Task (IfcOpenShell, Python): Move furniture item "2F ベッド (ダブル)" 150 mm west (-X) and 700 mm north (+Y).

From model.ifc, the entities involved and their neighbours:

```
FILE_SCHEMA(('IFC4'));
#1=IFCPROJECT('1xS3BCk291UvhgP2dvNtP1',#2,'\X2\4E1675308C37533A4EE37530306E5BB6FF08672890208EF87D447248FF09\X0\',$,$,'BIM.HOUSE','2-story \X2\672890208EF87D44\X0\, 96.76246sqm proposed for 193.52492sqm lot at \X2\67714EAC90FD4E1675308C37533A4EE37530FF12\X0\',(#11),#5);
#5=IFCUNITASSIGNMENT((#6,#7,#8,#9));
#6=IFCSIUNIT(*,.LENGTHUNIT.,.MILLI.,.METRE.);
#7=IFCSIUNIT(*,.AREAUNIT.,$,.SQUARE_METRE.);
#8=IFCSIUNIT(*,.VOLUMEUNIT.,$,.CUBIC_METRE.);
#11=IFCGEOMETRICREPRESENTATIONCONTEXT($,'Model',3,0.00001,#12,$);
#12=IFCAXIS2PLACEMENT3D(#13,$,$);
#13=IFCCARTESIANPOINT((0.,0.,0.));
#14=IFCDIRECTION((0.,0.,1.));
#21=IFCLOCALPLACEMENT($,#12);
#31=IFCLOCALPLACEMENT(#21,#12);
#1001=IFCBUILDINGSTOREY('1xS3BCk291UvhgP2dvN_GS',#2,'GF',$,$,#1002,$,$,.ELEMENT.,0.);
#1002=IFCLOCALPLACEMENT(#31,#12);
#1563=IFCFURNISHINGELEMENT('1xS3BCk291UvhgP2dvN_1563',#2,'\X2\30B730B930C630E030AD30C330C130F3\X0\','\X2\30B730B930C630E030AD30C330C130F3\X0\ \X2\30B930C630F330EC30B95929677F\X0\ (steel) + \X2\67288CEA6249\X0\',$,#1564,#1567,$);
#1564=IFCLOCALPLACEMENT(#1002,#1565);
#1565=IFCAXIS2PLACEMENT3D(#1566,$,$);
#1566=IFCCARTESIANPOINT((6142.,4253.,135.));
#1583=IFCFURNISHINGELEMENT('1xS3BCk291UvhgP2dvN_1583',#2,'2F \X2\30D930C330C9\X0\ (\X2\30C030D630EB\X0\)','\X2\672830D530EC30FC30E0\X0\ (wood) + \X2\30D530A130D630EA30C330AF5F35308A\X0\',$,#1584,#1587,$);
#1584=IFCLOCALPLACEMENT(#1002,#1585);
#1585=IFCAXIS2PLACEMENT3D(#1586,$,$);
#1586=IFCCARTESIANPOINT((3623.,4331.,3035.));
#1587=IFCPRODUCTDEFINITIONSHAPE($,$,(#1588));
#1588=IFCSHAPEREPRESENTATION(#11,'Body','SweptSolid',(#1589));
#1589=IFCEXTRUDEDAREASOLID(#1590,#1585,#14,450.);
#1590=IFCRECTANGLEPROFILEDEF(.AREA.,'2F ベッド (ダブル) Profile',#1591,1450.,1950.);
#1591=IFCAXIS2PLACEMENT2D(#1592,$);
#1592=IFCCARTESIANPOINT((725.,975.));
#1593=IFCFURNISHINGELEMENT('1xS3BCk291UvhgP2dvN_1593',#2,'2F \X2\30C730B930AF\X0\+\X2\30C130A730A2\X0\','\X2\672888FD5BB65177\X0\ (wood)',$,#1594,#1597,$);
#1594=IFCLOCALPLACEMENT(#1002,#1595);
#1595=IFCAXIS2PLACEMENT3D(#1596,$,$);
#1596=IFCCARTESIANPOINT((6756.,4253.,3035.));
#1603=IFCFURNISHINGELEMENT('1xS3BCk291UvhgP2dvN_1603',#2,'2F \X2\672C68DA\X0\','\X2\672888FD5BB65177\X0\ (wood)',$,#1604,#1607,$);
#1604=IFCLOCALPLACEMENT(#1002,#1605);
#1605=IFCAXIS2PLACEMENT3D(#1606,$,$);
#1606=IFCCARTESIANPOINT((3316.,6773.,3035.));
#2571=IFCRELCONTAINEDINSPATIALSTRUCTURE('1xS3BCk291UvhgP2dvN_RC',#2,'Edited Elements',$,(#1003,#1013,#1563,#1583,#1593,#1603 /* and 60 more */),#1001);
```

```python
import ifcopenshell
import ifcopenshell.api.geometry
import ifcopenshell.util.placement
import ifcopenshell.util.unit

model = ifcopenshell.open("model.ifc")
unit_scale = ifcopenshell.util.unit.calculate_unit_scale(model)

item = model.by_guid("1xS3BCk291UvhgP2dvN_1583")
matrix = ifcopenshell.util.placement.get_local_placement(item.ObjectPlacement)
matrix[0, 3] -= 0.15 / unit_scale
matrix[1, 3] += 0.7 / unit_scale
ifcopenshell.api.geometry.edit_object_placement(model, product=item, matrix=matrix, is_si=False)

print(ifcopenshell.util.placement.get_local_placement(item.ObjectPlacement).round(3) + 0.0)

model.write("model_updated.ifc")
```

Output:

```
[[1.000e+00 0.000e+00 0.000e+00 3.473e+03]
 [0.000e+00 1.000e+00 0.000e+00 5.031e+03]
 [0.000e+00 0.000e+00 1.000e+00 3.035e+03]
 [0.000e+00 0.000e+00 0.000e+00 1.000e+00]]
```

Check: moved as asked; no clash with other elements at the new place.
